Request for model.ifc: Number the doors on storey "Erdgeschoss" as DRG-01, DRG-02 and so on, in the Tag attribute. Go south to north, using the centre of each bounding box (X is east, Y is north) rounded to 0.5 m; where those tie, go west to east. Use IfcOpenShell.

First a look at what the model holds.

```python
import ifcopenshell
import ifcopenshell.util.element
import ifcopenshell.util.placement

model = ifcopenshell.open("model.ifc")
print(model.schema)
storey = next(s for s in model.by_type("IfcBuildingStorey") if s.Name == "Erdgeschoss")
doors = [e for e in ifcopenshell.util.element.get_decomposition(storey) if e.is_a("IfcDoor")]
for e in sorted(doors, key=lambda e: e.id()):
    origin = ifcopenshell.util.placement.get_local_placement(e.ObjectPlacement)[:3, 3]
    print(e.id(), e.Tag, e.Name, origin.round(2) + 0.0, sep=" | ")
```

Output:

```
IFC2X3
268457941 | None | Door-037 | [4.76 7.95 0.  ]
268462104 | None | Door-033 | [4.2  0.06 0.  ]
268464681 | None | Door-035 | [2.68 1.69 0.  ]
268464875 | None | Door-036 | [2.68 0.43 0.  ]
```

```python
import ifcopenshell
import ifcopenshell.geom
import ifcopenshell.util.element
import ifcopenshell.util.shape

model = ifcopenshell.open("model.ifc")
settings = ifcopenshell.geom.settings()
settings.set("use-world-coords", True)


def centre(element):
    shape = ifcopenshell.geom.create_shape(settings, element)
    return ifcopenshell.util.shape.get_bbox_centroid(shape.geometry)


storey = next(s for s in model.by_type("IfcBuildingStorey") if s.Name == "Erdgeschoss")
doors = [e for e in ifcopenshell.util.element.get_decomposition(storey) if e.is_a("IfcDoor")]

# Insertion points can sit at a corner or the storey origin, so sort by the geometry (in metres).
centres = {e: centre(e) for e in doors}
doors.sort(key=lambda e: (round(centres[e][1] / 0.5), centres[e][0]))

for i, e in enumerate(doors, start=1):
    number = f"DRG-{i:02d}"
    e.Tag = number
    print(e.id(), number)

model.write("model_edited.ifc")
```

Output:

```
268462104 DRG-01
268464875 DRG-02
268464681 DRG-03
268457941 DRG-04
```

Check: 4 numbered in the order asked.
